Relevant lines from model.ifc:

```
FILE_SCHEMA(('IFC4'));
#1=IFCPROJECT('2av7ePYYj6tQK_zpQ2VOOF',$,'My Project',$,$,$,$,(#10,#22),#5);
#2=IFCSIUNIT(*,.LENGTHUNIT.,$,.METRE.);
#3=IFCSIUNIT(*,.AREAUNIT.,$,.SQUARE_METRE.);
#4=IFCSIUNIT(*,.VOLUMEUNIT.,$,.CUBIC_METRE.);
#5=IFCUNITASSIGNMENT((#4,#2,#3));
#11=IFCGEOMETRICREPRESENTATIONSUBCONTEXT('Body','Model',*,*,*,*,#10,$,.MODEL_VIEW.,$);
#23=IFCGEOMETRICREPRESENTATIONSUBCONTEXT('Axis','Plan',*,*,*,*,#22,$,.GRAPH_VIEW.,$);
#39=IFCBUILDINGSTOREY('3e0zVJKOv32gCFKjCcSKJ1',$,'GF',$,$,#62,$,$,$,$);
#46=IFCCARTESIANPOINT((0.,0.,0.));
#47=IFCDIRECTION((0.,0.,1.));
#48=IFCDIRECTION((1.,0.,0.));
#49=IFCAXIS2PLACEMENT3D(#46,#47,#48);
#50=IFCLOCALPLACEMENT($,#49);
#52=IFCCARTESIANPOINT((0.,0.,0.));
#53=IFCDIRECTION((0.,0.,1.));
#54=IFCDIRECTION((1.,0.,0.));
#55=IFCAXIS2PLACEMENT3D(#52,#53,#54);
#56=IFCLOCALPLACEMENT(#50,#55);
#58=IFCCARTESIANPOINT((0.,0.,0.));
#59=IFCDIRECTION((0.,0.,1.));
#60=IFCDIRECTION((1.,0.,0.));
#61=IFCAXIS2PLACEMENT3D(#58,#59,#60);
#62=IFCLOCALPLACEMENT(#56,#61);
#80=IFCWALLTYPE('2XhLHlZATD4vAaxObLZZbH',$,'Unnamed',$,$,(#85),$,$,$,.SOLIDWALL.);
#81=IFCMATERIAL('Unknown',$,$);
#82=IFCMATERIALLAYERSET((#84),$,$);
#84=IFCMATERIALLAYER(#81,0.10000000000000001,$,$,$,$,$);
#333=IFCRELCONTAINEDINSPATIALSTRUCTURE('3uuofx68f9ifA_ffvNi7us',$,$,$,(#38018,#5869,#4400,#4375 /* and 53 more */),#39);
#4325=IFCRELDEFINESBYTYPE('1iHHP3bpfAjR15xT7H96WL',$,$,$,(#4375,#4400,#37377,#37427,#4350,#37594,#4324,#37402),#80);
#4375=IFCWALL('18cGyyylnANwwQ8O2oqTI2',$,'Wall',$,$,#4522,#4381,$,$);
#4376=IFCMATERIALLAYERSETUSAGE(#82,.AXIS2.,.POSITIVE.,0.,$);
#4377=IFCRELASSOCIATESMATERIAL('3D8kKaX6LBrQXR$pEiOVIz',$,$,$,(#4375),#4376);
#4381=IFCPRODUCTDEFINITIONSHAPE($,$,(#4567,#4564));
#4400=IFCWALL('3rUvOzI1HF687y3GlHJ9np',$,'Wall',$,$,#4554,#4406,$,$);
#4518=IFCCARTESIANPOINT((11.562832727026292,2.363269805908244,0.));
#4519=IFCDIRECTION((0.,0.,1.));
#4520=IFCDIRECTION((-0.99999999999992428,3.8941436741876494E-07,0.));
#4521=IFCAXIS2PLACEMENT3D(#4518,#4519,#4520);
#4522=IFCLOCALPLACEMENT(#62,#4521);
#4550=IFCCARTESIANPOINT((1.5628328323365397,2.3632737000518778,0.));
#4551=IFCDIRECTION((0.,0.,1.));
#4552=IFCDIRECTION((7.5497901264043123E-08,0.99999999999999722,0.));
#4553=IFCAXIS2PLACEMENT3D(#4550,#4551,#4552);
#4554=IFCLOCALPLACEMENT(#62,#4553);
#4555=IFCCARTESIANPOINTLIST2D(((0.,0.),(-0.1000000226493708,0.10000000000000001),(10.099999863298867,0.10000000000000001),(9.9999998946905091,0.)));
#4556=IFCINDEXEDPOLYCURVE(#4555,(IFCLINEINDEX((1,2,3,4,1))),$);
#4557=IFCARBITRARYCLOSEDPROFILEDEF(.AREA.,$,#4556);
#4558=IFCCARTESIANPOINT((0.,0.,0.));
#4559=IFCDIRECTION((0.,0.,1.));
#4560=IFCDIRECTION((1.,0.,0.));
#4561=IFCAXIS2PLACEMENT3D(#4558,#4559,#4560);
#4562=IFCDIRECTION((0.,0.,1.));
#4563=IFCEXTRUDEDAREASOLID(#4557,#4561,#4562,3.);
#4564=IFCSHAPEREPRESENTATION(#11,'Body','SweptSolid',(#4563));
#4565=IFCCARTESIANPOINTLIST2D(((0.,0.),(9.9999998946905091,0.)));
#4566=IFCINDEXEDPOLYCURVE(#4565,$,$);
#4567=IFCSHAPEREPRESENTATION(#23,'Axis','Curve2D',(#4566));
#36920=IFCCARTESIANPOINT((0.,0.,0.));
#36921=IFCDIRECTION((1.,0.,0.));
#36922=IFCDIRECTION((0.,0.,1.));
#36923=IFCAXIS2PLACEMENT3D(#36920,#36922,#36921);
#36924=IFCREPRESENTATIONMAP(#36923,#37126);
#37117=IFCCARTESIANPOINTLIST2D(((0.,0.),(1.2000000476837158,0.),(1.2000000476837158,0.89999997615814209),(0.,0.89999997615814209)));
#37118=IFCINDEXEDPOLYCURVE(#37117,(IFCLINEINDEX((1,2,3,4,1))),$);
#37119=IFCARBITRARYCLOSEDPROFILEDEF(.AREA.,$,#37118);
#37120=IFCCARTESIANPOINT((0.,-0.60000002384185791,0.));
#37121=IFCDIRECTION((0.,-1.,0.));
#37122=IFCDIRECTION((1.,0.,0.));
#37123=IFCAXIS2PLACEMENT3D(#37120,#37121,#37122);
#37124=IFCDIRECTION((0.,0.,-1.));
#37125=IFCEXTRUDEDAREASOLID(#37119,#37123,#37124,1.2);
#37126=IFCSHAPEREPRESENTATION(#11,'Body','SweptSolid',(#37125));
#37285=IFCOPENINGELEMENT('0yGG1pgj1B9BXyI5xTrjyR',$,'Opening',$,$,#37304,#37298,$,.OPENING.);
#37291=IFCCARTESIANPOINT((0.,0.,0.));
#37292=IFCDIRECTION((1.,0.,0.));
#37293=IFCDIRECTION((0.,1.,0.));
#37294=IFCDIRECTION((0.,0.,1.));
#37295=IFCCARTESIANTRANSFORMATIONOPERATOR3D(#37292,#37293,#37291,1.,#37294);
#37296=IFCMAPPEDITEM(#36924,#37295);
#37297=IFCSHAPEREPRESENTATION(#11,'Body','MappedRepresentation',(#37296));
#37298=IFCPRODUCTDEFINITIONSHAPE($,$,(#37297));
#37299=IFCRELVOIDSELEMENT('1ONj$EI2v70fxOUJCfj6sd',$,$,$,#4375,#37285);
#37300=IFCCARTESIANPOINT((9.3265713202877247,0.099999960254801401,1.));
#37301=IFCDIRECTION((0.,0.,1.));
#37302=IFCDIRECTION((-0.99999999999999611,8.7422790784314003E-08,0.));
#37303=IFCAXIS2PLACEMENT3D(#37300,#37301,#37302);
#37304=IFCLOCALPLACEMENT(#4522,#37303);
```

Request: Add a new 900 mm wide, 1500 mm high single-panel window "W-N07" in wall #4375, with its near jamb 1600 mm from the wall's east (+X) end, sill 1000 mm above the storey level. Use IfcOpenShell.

```python
import numpy as np
import ifcopenshell
import ifcopenshell.api.feature
import ifcopenshell.api.geometry
import ifcopenshell.api.root
import ifcopenshell.api.spatial
import ifcopenshell.geom
import ifcopenshell.util.element
import ifcopenshell.util.placement
import ifcopenshell.util.representation
import ifcopenshell.util.shape
import ifcopenshell.util.unit

model = ifcopenshell.open("model.ifc")
unit_scale = ifcopenshell.util.unit.calculate_unit_scale(model)
settings = ifcopenshell.geom.settings()


def volume(element):
    """Net volume in cubic metres, openings subtracted."""
    shape = ifcopenshell.geom.create_shape(settings, element)
    return ifcopenshell.util.shape.get_volume(shape.geometry)


wall = model.by_guid("18cGyyylnANwwQ8O2oqTI2")
storey = ifcopenshell.util.element.get_container(wall, ifc_class="IfcBuildingStorey")
context = ifcopenshell.util.representation.get_context(model, "Model", "Body", "MODEL_VIEW")
before = volume(wall)

width, height, from_end, sill = 0.9, 1.5, 1.6, 1  # metres

# The wall runs along its own X axis, and the end named is its -X end.
wall_shape = ifcopenshell.geom.create_shape(settings, wall)
x, y, z = ifcopenshell.util.shape.get_vertices(wall_shape.geometry).T
start = x.min() + from_end
face, thickness = float(y.min()), float(y.max() - y.min())
wall_matrix = ifcopenshell.util.placement.get_local_placement(wall.ObjectPlacement)
level = ifcopenshell.util.placement.get_local_placement(storey.ObjectPlacement)[2, 3]


def in_wall(x, y):
    """Placement at x, y metres in the wall's axes, at sill height."""
    matrix = wall_matrix.copy()
    matrix[:, 3] = wall_matrix @ np.array([x / unit_scale, y / unit_scale, 0.0, 1.0])
    matrix[2, 3] = level + sill / unit_scale
    return matrix


# Opening: a box that overshoots both wall faces by 50 mm.
opening = ifcopenshell.api.root.create_entity(model, ifc_class="IfcOpeningElement", predefined_type="OPENING")
box = ifcopenshell.api.geometry.add_wall_representation(
    model, context=context, length=width, height=height, thickness=thickness + 0.1
)
ifcopenshell.api.geometry.assign_representation(model, product=opening, representation=box)
ifcopenshell.api.geometry.edit_object_placement(model, product=opening, matrix=in_wall(start, face - 0.05), is_si=False)
ifcopenshell.api.feature.add_feature(model, feature=opening, element=wall)

window = ifcopenshell.api.root.create_entity(model, ifc_class="IfcWindow", name="W-N07", predefined_type="WINDOW")
window.OverallWidth, window.OverallHeight = width / unit_scale, height / unit_scale
window.PartitioningType = "SINGLE_PANEL"
body = ifcopenshell.api.geometry.add_window_representation(
    model,
    context=context,
    overall_width=window.OverallWidth,
    overall_height=window.OverallHeight,
    partition_type="SINGLE_PANEL",
)
ifcopenshell.api.geometry.assign_representation(model, product=window, representation=body)
ifcopenshell.api.spatial.assign_container(model, products=[window], relating_structure=storey)
ifcopenshell.api.feature.add_filling(model, opening=opening, element=window)

# Centre the window in the wall's thickness.
ifcopenshell.api.geometry.edit_object_placement(model, product=window, matrix=in_wall(start, face), is_si=False)
window_shape = ifcopenshell.geom.create_shape(settings, window)
depth = ifcopenshell.util.shape.get_vertices(window_shape.geometry)[:, 1]
offset = face + thickness / 2 - (depth.min() + depth.max()) / 2
ifcopenshell.api.geometry.edit_object_placement(model, product=window, matrix=in_wall(start, offset), is_si=False)

after = volume(wall)

print(f"wall volume {before:.3f} -> {after:.3f} m3")

model.write("model_updated.ifc")
```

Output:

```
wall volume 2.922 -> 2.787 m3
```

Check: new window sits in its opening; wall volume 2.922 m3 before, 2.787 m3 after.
